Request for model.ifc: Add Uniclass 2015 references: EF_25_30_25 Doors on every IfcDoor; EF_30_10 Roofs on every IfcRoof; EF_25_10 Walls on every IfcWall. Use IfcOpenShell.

First a look at what the model holds.

```python
import ifcopenshell

model = ifcopenshell.open("model.ifc")
print(model.schema)
print("classifications:", [c.Name for c in model.by_type("IfcClassification")])
for ifc_class in ("IfcDoor", "IfcRoof", "IfcStair", "IfcWall", "IfcWindow"):
    print(ifc_class, len(model.by_type(ifc_class)))
```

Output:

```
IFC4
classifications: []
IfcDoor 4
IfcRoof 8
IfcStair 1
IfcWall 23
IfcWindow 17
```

```python
import ifcopenshell
import ifcopenshell.api.classification

model = ifcopenshell.open("model.ifc")

system = ifcopenshell.api.classification.add_classification(model, classification="Uniclass 2015")

codes = {
    "IfcDoor": ("EF_25_30_25", "Doors"),
    "IfcRoof": ("EF_30_10", "Roofs"),
    "IfcWall": ("EF_25_10", "Walls"),
}
for ifc_class, (code, name) in codes.items():
    products = model.by_type(ifc_class)
    ifcopenshell.api.classification.add_reference(
        model, products=products, classification=system, identification=code, name=name
    )
    print(code, len(products))

model.write("model_v2.ifc")
```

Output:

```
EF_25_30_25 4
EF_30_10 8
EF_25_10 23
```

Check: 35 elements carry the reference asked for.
